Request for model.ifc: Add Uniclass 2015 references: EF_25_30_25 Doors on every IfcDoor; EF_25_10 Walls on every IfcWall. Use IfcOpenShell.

First a look at what the model holds.

```python
import ifcopenshell

model = ifcopenshell.open("model.ifc")
print(model.schema)
print("classifications:", [c.Name for c in model.by_type("IfcClassification")])
for ifc_class in ("IfcDoor", "IfcRoof", "IfcStair", "IfcWall", "IfcWindow"):
    print(ifc_class, len(model.by_type(ifc_class)))
```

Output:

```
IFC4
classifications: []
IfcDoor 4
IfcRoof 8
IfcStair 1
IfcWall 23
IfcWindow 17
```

```python
import ifcopenshell
import ifcopenshell.api.classification

model = ifcopenshell.open("model.ifc")

system = ifcopenshell.api.classification.add_classification(model, classification="Uniclass 2015")

codes = {
    "IfcDoor": ("EF_25_30_25", "Doors"),
    "IfcWall": ("EF_25_10", "Walls"),
}
for ifc_class, (code, name) in codes.items():
    products = model.by_type(ifc_class)
    ifcopenshell.api.classification.add_reference(
        model, products=products, classification=system, identification=code, name=name
    )
    print(code, len(products))

model.write("model_updated.ifc")
```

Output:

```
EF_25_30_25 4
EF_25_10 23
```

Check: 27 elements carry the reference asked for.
